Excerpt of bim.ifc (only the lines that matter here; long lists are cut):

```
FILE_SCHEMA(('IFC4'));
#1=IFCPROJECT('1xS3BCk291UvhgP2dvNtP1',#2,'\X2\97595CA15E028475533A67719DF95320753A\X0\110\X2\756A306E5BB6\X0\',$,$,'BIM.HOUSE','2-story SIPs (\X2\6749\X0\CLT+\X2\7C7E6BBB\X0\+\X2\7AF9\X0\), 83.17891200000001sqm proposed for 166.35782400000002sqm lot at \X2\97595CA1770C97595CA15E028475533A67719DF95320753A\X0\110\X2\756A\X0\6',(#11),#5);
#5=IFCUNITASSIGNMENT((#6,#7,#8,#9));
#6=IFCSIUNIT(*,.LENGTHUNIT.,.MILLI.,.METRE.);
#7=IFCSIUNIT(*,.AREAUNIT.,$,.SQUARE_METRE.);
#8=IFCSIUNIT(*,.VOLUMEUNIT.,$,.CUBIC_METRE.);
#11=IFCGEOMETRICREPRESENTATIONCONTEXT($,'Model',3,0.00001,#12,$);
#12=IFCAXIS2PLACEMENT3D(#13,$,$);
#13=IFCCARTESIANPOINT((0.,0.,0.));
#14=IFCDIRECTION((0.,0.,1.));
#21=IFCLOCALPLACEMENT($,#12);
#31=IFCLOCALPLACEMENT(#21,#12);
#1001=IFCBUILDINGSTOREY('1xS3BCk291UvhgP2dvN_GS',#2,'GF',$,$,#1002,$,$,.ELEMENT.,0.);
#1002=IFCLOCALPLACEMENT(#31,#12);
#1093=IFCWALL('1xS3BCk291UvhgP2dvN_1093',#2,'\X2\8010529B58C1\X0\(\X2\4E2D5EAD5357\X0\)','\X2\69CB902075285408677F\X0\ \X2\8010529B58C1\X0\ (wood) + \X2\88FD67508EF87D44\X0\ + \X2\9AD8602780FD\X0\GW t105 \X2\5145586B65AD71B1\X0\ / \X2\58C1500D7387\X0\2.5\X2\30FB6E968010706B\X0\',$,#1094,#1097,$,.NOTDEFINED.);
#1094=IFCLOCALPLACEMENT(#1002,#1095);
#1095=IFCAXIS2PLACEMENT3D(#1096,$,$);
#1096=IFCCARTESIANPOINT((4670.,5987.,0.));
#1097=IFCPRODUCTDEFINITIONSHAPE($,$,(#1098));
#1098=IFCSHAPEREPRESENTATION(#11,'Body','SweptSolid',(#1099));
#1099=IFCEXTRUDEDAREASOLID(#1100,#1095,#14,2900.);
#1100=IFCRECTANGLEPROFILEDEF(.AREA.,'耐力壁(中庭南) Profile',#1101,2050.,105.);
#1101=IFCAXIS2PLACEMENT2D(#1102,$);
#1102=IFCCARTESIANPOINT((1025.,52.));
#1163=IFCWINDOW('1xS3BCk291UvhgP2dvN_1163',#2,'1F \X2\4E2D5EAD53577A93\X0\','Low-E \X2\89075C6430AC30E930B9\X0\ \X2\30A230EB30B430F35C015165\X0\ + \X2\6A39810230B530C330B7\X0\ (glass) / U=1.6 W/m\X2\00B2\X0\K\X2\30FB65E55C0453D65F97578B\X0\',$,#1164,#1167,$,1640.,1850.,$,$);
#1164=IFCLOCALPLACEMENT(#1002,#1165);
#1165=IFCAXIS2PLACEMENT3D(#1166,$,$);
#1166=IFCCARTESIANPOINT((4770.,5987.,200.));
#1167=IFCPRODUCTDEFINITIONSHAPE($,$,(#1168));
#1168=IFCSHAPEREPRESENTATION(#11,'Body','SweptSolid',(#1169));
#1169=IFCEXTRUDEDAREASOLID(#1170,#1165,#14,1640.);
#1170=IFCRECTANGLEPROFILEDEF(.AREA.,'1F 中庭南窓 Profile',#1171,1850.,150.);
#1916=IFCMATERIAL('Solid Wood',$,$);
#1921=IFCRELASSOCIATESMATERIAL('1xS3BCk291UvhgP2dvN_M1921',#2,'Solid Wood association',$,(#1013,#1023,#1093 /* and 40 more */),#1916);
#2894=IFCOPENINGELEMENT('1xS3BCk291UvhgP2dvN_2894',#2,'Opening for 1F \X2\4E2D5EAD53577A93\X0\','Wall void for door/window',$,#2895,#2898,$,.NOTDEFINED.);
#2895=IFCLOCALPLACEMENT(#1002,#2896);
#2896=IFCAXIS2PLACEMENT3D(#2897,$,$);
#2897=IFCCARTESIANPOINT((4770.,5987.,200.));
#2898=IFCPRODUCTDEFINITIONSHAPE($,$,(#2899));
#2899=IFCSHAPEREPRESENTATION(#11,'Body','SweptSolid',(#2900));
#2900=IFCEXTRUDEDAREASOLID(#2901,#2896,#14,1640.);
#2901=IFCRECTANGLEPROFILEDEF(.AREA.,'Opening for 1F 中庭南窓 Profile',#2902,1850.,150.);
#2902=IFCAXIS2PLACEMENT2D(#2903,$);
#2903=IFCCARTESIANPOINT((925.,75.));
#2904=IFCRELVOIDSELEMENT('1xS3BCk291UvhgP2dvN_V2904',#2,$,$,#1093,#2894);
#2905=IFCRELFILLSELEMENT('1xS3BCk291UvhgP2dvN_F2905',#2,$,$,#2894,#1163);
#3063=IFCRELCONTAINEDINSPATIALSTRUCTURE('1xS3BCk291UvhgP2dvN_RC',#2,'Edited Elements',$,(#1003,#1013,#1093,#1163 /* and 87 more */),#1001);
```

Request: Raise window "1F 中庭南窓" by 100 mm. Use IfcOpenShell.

```python
import numpy as np
import ifcopenshell
import ifcopenshell.api.geometry
import ifcopenshell.util.placement
import ifcopenshell.util.unit

model = ifcopenshell.open("bim.ifc")
unit_scale = ifcopenshell.util.unit.calculate_unit_scale(model)

window = model.by_guid("1xS3BCk291UvhgP2dvN_1163")
opening = window.FillsVoids[0].RelatingOpeningElement
dz = 0.1 / unit_scale

shift = np.array([0.0, 0.0, dz])
# The window is not placed relative to its opening, so move both.
for product in (opening, window):
    matrix = ifcopenshell.util.placement.get_local_placement(product.ObjectPlacement)
    matrix[:3, 3] += shift
    ifcopenshell.api.geometry.edit_object_placement(model, product=product, matrix=matrix, is_si=False)

print(f"moved by {dz * unit_scale:+.3f} m")

model.write("bim_v2.ifc")
```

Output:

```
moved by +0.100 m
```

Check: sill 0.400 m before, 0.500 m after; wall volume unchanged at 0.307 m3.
